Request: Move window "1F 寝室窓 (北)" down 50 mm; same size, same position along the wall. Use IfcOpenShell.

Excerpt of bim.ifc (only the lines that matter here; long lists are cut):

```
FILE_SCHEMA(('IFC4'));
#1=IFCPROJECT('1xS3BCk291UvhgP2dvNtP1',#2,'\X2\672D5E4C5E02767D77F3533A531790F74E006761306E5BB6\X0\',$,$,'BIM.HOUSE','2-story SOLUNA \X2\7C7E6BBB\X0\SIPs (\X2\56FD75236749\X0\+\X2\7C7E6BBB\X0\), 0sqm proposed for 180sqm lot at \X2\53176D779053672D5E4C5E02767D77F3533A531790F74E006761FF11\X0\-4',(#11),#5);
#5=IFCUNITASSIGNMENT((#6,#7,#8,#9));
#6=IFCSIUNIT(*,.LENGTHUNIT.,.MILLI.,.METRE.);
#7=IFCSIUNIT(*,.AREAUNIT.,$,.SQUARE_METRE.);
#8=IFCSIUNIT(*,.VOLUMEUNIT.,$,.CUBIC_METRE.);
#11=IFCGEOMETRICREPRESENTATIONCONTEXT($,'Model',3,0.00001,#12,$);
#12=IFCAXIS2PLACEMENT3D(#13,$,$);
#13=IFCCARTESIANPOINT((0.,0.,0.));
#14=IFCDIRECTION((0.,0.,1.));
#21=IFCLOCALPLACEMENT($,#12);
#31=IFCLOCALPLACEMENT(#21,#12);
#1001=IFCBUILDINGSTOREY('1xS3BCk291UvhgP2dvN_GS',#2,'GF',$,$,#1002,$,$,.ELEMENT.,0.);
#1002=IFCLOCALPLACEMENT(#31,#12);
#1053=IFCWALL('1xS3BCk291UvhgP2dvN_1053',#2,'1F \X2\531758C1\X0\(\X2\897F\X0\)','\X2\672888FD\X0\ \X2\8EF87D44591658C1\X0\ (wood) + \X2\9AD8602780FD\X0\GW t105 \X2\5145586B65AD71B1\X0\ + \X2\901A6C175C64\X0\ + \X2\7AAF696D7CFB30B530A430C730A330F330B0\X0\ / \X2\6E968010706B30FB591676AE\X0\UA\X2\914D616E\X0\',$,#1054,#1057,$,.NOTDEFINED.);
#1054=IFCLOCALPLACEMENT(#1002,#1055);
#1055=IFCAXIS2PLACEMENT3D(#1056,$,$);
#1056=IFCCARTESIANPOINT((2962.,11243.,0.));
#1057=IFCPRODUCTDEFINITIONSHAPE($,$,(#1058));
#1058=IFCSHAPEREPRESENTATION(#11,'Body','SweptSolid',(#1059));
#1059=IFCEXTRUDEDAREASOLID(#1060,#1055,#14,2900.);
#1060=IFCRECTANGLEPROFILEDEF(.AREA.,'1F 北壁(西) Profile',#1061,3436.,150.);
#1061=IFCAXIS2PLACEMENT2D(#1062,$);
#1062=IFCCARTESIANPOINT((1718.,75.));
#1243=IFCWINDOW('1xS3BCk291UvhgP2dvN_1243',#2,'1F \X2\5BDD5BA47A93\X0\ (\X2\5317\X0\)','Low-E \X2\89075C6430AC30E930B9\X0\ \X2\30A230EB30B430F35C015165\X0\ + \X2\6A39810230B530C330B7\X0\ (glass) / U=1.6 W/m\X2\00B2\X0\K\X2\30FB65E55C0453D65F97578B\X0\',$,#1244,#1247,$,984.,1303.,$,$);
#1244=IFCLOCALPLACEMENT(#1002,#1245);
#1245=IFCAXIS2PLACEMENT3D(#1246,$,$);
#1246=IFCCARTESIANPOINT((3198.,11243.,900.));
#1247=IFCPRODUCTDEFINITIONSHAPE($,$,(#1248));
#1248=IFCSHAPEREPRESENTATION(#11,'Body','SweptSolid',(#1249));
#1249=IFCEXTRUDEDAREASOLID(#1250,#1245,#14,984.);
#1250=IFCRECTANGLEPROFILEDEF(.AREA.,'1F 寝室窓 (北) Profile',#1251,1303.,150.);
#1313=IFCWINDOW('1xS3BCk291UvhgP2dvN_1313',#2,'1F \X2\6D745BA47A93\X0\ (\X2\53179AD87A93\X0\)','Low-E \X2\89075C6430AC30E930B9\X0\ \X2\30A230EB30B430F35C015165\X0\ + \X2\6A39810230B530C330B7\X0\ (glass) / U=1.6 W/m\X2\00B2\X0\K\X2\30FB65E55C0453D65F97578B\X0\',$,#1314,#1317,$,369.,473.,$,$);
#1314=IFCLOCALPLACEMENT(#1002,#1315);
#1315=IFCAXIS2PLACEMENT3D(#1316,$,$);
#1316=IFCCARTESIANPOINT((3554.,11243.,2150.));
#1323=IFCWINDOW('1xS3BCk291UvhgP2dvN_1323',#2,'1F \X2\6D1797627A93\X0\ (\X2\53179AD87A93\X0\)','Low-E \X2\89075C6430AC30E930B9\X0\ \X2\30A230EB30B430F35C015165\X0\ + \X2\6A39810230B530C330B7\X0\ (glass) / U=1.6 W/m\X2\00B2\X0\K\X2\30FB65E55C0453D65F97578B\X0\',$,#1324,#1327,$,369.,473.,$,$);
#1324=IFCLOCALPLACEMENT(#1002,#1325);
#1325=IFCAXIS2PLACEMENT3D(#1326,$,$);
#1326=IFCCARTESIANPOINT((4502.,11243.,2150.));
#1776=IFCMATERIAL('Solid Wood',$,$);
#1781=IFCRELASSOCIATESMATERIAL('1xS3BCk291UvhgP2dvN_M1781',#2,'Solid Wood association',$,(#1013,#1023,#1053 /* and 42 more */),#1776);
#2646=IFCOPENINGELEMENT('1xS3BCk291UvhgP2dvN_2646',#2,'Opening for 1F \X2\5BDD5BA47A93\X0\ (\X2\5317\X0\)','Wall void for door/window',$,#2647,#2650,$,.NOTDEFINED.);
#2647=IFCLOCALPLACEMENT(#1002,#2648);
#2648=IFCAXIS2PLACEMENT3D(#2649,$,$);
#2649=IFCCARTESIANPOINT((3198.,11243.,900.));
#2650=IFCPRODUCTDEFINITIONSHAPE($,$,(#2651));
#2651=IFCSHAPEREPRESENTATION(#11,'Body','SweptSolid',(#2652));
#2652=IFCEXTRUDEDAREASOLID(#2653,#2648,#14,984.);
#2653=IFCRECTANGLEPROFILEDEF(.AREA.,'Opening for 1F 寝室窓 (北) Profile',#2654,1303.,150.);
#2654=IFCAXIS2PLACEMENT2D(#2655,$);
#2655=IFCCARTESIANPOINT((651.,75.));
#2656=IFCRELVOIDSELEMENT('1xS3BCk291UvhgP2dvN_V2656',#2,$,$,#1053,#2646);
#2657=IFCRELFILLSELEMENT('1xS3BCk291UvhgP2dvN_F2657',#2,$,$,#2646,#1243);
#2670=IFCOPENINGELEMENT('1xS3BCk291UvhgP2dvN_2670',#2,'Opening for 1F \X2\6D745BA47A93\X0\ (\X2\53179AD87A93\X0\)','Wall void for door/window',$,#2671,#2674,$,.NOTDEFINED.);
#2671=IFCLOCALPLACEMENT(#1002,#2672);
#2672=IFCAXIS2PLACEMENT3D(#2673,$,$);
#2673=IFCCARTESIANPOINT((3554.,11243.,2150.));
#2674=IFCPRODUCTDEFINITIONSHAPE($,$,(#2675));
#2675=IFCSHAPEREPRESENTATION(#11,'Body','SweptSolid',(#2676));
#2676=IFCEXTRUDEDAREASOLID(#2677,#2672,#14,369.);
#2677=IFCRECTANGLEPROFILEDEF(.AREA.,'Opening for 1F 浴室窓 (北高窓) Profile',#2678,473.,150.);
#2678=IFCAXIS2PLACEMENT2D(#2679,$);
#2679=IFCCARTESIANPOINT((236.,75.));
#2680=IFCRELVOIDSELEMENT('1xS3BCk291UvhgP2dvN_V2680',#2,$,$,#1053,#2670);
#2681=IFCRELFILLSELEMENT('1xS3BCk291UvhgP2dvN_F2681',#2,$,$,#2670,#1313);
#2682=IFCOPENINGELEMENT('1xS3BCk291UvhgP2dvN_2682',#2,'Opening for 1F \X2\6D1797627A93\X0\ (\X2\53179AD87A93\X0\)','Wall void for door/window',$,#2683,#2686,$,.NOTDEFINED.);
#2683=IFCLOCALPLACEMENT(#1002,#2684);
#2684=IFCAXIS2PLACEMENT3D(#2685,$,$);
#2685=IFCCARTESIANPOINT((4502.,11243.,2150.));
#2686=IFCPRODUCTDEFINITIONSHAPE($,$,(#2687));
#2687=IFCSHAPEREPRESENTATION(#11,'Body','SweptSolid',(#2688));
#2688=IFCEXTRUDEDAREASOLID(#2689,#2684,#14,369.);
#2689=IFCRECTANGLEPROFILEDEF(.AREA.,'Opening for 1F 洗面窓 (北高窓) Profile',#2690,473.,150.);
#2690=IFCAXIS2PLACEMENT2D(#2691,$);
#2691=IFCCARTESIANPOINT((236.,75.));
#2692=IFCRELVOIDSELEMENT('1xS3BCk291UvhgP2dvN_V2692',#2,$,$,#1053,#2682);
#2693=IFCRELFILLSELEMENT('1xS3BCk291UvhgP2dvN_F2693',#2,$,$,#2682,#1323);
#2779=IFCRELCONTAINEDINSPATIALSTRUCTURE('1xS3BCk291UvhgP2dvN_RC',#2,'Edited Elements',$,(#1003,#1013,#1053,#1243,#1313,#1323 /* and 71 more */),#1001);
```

```python
import numpy as np
import ifcopenshell
import ifcopenshell.api.geometry
import ifcopenshell.util.placement
import ifcopenshell.util.unit

model = ifcopenshell.open("bim.ifc")
unit_scale = ifcopenshell.util.unit.calculate_unit_scale(model)

window = model.by_guid("1xS3BCk291UvhgP2dvN_1243")
opening = window.FillsVoids[0].RelatingOpeningElement
dz = -50.0

shift = np.array([0.0, 0.0, dz])
# The window is not placed relative to its opening, so move both.
for product in (opening, window):
    matrix = ifcopenshell.util.placement.get_local_placement(product.ObjectPlacement)
    matrix[:3, 3] += shift
    ifcopenshell.api.geometry.edit_object_placement(model, product=product, matrix=matrix, is_si=False)

print(f"moved by {dz * unit_scale:+.3f} m")

model.write("bim_updated.ifc")
```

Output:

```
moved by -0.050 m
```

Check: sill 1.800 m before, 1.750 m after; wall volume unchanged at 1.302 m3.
